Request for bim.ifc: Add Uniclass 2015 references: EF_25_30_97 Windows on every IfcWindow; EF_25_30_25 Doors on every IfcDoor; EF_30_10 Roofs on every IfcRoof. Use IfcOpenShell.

First a look at what the model holds.

```python
import ifcopenshell

model = ifcopenshell.open("bim.ifc")
print(model.schema)
print("classifications:", [c.Name for c in model.by_type("IfcClassification")])
for ifc_class in ("IfcDoor", "IfcRoof", "IfcStair", "IfcWall", "IfcWindow"):
    print(ifc_class, len(model.by_type(ifc_class)))
```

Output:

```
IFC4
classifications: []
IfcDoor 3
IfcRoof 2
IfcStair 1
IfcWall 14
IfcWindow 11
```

```python
import ifcopenshell
import ifcopenshell.api.classification

model = ifcopenshell.open("bim.ifc")

system = ifcopenshell.api.classification.add_classification(model, classification="Uniclass 2015")

codes = {
    "IfcWindow": ("EF_25_30_97", "Windows"),
    "IfcDoor": ("EF_25_30_25", "Doors"),
    "IfcRoof": ("EF_30_10", "Roofs"),
}
for ifc_class, (code, name) in codes.items():
    products = model.by_type(ifc_class)
    ifcopenshell.api.classification.add_reference(
        model, products=products, classification=system, identification=code, name=name
    )
    print(code, len(products))

model.write("bim_updated.ifc")
```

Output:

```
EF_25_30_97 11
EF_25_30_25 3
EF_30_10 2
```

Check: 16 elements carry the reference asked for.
